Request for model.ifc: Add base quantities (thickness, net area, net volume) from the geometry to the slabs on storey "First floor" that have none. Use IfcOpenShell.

First a look at what the model holds.

```python
import ifcopenshell
import ifcopenshell.util.element
import ifcopenshell.util.unit

model = ifcopenshell.open("model.ifc")
print(model.schema)
for unit_type in ("LENGTHUNIT", "AREAUNIT", "VOLUMEUNIT"):
    print(unit_type, ifcopenshell.util.unit.calculate_unit_scale(model, unit_type))
storey = next(s for s in model.by_type("IfcBuildingStorey") if s.Name == "First floor")
slabs = [e for e in ifcopenshell.util.element.get_decomposition(storey) if e.is_a("IfcSlab")]
for e in sorted(slabs, key=lambda e: e.id()):
    print(e.id(), e.is_a(), e.Name, list(ifcopenshell.util.element.get_psets(e, qtos_only=True)), sep=" | ")
```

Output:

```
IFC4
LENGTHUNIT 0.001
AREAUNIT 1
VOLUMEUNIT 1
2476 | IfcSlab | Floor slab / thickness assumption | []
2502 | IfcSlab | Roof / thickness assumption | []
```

```python
import ifcopenshell
import ifcopenshell.api.pset
import ifcopenshell.geom
import ifcopenshell.util.element
import ifcopenshell.util.shape
import ifcopenshell.util.unit

model = ifcopenshell.open("model.ifc")
unit_scale = ifcopenshell.util.unit.calculate_unit_scale(model)
area_scale = ifcopenshell.util.unit.calculate_unit_scale(model, "AREAUNIT")
volume_scale = ifcopenshell.util.unit.calculate_unit_scale(model, "VOLUMEUNIT")
settings = ifcopenshell.geom.settings()

storey = next(s for s in model.by_type("IfcBuildingStorey") if s.Name == "First floor")
slabs = [e for e in ifcopenshell.util.element.get_decomposition(storey) if e.is_a("IfcSlab")]

for e in sorted(slabs, key=lambda e: e.id()):
    if ifcopenshell.util.element.get_psets(e, qtos_only=True, should_inherit=False):
        continue
    # Geometry comes back in metres, in the element's own axes.
    shape = ifcopenshell.geom.create_shape(settings, e)
    values = {
        "Width": ifcopenshell.util.shape.get_z(shape.geometry) / unit_scale,
        "NetArea": ifcopenshell.util.shape.get_footprint_area(shape.geometry) / area_scale,
        "NetVolume": ifcopenshell.util.shape.get_volume(shape.geometry) / volume_scale,
    }
    qto = ifcopenshell.api.pset.add_qto(model, product=e, name="Qto_SlabBaseQuantities")
    ifcopenshell.api.pset.edit_qto(model, qto=qto, properties=values)
    print(e.id(), {k: round(v, 3) for k, v in values.items()})

model.write("model_edited.ifc")
```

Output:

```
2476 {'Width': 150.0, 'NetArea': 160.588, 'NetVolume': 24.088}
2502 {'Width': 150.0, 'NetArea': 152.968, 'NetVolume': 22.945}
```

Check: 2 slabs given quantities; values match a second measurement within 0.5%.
